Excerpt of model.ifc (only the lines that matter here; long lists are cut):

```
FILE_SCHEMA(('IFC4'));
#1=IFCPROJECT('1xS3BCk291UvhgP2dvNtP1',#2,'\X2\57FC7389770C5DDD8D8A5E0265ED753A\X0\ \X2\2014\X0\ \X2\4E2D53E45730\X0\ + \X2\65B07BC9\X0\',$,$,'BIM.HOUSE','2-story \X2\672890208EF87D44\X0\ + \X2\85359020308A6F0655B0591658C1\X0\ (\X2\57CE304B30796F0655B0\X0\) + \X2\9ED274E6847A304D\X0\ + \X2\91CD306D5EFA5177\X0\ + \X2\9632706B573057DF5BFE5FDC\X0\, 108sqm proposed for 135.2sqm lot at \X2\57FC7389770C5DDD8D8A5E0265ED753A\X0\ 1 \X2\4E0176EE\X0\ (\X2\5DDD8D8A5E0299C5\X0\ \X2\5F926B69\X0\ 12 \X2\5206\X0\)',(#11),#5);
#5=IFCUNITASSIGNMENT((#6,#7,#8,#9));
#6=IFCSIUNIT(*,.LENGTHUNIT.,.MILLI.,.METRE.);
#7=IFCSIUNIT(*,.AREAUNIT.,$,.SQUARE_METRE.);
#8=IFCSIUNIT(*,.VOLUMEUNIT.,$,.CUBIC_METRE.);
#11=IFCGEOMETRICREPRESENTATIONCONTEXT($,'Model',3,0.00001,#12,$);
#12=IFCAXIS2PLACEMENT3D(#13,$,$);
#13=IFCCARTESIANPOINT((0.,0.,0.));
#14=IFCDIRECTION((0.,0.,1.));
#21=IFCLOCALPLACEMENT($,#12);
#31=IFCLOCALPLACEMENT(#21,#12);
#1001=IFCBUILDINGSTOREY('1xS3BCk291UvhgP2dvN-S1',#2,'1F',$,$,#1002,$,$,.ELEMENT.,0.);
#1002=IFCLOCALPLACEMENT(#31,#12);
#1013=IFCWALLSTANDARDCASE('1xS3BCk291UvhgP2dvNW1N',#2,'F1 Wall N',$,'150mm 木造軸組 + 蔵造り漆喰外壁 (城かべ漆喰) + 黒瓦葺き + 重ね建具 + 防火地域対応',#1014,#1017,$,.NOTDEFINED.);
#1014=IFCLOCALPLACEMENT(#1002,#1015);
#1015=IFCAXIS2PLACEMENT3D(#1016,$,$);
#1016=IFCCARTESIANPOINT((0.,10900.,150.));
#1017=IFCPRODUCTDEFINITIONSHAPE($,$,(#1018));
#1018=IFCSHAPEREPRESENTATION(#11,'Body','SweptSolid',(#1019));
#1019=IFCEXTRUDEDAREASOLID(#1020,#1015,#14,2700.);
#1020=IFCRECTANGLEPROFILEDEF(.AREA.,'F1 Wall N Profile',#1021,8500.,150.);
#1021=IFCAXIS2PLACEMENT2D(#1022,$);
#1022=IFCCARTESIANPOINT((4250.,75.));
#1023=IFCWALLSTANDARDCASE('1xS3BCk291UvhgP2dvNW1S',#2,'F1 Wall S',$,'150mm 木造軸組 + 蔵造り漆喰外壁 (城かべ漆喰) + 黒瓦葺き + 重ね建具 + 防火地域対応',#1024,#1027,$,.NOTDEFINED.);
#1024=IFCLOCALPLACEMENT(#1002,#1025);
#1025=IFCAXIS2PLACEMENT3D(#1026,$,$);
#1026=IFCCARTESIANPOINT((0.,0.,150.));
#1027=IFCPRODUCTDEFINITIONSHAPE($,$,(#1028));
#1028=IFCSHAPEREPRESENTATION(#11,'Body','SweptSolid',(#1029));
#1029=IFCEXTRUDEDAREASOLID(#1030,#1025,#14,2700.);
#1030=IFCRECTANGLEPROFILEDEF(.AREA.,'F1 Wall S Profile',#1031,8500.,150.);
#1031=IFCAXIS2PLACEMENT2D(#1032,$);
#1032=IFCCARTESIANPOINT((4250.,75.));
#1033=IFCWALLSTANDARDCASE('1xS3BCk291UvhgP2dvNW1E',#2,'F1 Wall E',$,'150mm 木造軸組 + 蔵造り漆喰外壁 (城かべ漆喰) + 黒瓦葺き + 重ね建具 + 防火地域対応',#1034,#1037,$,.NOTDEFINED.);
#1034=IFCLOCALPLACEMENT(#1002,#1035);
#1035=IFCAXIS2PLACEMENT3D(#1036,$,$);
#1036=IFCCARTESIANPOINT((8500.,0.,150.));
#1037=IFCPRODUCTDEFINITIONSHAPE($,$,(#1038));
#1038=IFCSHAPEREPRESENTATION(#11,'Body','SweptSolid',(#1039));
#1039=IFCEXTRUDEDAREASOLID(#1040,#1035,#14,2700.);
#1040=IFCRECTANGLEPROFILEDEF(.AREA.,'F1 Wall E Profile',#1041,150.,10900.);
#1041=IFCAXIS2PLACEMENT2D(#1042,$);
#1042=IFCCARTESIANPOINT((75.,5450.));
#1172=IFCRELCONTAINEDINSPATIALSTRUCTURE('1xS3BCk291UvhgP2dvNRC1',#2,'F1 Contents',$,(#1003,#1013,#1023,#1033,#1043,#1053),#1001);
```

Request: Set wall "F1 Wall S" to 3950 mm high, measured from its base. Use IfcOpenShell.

```python
import ifcopenshell
import ifcopenshell.geom
import ifcopenshell.util.shape
import ifcopenshell.util.unit

model = ifcopenshell.open("model.ifc")
unit_scale = ifcopenshell.util.unit.calculate_unit_scale(model)
settings = ifcopenshell.geom.settings()


def volume(element):
    """Net volume in cubic metres, openings subtracted."""
    shape = ifcopenshell.geom.create_shape(settings, element)
    return ifcopenshell.util.shape.get_volume(shape.geometry)


wall = model.by_guid("1xS3BCk291UvhgP2dvNW1S")
before = volume(wall)

body = next(r for r in wall.Representation.Representations if r.RepresentationIdentifier == "Body")
solid = body.Items[0]
old_height = solid.Depth
solid.Depth = 3.95 / unit_scale
after = volume(wall)

print(f"height {old_height:g} -> {solid.Depth:g}, volume {before:.3f} -> {after:.3f} m3")

model.write("model_edited.ifc")
```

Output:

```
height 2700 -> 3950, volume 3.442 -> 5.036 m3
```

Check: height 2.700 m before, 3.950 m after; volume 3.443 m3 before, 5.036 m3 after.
